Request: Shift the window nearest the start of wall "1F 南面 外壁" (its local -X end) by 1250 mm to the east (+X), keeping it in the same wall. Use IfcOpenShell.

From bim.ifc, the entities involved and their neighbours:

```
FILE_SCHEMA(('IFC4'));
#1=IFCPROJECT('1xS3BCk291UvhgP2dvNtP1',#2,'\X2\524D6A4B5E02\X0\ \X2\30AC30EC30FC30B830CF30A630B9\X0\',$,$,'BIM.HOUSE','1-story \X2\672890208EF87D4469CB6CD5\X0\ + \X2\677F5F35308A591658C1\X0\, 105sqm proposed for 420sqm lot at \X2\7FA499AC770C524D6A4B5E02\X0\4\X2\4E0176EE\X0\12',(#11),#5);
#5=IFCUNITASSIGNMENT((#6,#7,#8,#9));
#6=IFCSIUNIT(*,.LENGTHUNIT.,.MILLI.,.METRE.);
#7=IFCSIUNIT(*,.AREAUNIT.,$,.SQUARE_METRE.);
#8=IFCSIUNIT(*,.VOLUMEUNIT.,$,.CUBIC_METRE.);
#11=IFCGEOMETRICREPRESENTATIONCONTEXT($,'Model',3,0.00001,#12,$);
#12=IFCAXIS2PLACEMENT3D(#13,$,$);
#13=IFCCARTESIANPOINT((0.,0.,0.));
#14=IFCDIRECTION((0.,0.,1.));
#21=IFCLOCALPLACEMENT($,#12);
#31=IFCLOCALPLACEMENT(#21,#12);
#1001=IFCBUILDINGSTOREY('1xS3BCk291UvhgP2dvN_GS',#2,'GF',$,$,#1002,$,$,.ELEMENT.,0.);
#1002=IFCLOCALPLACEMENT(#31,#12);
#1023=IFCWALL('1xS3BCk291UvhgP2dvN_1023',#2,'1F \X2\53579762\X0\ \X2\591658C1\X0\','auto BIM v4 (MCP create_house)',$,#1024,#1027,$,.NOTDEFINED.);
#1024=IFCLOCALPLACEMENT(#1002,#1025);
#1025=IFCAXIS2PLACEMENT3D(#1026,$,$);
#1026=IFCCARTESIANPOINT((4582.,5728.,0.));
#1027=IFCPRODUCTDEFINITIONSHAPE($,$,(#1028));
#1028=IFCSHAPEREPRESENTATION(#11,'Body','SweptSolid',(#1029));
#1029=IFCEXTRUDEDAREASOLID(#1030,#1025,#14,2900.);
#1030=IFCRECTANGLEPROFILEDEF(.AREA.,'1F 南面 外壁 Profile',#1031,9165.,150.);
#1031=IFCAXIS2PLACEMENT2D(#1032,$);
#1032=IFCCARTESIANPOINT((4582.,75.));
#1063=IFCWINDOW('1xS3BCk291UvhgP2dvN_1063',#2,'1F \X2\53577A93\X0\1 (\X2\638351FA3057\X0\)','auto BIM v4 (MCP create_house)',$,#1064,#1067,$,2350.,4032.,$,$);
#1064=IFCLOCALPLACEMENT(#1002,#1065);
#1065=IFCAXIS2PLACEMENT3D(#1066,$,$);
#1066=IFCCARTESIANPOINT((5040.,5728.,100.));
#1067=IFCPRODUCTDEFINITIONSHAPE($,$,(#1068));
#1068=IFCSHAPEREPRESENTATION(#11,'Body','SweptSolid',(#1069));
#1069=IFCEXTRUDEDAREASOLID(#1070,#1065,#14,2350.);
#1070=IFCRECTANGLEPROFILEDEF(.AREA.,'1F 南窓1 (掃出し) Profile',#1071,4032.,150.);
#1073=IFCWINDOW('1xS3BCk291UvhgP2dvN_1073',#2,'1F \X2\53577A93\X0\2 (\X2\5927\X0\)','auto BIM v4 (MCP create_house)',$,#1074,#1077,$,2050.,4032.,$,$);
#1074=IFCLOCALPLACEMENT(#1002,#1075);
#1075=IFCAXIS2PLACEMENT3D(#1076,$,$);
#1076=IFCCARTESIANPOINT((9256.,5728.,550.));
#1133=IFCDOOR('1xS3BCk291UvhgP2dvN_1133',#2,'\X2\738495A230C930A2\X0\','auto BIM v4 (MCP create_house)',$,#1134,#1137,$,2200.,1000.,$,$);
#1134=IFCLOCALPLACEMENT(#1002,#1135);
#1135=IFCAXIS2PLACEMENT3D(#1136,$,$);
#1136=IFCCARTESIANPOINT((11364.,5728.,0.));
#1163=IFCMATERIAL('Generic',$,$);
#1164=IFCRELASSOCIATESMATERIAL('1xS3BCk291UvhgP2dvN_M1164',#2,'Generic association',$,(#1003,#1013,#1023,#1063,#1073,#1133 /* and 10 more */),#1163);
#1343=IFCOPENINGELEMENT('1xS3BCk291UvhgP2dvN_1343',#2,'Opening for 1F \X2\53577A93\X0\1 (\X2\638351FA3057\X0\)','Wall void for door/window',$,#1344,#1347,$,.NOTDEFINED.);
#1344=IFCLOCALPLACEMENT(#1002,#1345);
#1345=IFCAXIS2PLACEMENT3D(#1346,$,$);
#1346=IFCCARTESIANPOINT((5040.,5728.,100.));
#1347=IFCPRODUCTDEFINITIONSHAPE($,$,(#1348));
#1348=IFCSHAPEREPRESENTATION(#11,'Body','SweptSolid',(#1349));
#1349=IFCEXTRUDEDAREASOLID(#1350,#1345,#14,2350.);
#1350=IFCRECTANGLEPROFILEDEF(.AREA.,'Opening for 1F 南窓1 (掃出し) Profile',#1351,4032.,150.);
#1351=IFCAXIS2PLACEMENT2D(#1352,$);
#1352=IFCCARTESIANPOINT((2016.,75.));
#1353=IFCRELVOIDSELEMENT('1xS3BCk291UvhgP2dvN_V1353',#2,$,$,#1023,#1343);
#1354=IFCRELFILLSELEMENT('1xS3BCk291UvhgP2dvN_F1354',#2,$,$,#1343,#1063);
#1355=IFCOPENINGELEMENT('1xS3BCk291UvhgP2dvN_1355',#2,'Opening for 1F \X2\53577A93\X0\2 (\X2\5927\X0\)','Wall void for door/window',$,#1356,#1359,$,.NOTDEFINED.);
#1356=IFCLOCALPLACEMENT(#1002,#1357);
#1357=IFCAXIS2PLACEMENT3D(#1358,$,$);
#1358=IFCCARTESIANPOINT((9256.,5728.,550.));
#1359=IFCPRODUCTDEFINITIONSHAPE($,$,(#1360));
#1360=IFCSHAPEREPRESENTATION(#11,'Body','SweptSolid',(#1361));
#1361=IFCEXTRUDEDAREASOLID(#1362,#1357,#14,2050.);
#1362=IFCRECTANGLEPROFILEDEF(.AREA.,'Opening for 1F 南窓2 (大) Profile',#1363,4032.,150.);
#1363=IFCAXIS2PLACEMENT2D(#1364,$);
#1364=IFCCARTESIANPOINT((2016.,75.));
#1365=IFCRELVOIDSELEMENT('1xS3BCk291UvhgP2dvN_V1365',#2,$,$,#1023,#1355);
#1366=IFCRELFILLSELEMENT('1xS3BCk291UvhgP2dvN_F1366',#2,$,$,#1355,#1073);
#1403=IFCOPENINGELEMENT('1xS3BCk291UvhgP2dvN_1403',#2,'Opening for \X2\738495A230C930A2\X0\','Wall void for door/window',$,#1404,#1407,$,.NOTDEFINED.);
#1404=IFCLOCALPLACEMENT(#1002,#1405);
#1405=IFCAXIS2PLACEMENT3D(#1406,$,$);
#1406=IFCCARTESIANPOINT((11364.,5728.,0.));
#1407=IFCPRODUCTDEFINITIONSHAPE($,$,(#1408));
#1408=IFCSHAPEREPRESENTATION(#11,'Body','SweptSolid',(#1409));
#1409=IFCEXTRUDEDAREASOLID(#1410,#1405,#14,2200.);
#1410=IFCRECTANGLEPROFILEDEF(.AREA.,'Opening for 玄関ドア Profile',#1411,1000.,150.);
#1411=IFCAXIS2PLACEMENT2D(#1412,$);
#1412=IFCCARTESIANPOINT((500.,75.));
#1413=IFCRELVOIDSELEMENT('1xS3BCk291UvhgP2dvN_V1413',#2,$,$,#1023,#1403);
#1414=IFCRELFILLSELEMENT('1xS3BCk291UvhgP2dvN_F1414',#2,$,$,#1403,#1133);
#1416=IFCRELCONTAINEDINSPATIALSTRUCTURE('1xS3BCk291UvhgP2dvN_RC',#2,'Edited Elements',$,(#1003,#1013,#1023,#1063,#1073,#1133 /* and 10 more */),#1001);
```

```python
import ifcopenshell
import ifcopenshell.api.geometry
import ifcopenshell.util.placement
import ifcopenshell.util.unit

model = ifcopenshell.open("bim.ifc")
unit_scale = ifcopenshell.util.unit.calculate_unit_scale(model)

window = model.by_id(1063)
opening = window.FillsVoids[0].RelatingOpeningElement
wall = opening.VoidsElements[0].RelatingBuildingElement

wall_matrix = ifcopenshell.util.placement.get_local_placement(wall.ObjectPlacement)
shift = wall_matrix[:3, 0] * 1.25 / unit_scale
before = ifcopenshell.util.placement.get_local_placement(window.ObjectPlacement)[:3, 3].copy()

# The window is not placed relative to its opening, so move both.
for product in (opening, window):
    matrix = ifcopenshell.util.placement.get_local_placement(product.ObjectPlacement)
    matrix[:3, 3] += shift
    ifcopenshell.api.geometry.edit_object_placement(model, product=product, matrix=matrix, is_si=False)

after = ifcopenshell.util.placement.get_local_placement(window.ObjectPlacement)[:3, 3]
print("window moved by", (after - before).round(3) + 0.0)

model.write("bim_v2.ifc")
```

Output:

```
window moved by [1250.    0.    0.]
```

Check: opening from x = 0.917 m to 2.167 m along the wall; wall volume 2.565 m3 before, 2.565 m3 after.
